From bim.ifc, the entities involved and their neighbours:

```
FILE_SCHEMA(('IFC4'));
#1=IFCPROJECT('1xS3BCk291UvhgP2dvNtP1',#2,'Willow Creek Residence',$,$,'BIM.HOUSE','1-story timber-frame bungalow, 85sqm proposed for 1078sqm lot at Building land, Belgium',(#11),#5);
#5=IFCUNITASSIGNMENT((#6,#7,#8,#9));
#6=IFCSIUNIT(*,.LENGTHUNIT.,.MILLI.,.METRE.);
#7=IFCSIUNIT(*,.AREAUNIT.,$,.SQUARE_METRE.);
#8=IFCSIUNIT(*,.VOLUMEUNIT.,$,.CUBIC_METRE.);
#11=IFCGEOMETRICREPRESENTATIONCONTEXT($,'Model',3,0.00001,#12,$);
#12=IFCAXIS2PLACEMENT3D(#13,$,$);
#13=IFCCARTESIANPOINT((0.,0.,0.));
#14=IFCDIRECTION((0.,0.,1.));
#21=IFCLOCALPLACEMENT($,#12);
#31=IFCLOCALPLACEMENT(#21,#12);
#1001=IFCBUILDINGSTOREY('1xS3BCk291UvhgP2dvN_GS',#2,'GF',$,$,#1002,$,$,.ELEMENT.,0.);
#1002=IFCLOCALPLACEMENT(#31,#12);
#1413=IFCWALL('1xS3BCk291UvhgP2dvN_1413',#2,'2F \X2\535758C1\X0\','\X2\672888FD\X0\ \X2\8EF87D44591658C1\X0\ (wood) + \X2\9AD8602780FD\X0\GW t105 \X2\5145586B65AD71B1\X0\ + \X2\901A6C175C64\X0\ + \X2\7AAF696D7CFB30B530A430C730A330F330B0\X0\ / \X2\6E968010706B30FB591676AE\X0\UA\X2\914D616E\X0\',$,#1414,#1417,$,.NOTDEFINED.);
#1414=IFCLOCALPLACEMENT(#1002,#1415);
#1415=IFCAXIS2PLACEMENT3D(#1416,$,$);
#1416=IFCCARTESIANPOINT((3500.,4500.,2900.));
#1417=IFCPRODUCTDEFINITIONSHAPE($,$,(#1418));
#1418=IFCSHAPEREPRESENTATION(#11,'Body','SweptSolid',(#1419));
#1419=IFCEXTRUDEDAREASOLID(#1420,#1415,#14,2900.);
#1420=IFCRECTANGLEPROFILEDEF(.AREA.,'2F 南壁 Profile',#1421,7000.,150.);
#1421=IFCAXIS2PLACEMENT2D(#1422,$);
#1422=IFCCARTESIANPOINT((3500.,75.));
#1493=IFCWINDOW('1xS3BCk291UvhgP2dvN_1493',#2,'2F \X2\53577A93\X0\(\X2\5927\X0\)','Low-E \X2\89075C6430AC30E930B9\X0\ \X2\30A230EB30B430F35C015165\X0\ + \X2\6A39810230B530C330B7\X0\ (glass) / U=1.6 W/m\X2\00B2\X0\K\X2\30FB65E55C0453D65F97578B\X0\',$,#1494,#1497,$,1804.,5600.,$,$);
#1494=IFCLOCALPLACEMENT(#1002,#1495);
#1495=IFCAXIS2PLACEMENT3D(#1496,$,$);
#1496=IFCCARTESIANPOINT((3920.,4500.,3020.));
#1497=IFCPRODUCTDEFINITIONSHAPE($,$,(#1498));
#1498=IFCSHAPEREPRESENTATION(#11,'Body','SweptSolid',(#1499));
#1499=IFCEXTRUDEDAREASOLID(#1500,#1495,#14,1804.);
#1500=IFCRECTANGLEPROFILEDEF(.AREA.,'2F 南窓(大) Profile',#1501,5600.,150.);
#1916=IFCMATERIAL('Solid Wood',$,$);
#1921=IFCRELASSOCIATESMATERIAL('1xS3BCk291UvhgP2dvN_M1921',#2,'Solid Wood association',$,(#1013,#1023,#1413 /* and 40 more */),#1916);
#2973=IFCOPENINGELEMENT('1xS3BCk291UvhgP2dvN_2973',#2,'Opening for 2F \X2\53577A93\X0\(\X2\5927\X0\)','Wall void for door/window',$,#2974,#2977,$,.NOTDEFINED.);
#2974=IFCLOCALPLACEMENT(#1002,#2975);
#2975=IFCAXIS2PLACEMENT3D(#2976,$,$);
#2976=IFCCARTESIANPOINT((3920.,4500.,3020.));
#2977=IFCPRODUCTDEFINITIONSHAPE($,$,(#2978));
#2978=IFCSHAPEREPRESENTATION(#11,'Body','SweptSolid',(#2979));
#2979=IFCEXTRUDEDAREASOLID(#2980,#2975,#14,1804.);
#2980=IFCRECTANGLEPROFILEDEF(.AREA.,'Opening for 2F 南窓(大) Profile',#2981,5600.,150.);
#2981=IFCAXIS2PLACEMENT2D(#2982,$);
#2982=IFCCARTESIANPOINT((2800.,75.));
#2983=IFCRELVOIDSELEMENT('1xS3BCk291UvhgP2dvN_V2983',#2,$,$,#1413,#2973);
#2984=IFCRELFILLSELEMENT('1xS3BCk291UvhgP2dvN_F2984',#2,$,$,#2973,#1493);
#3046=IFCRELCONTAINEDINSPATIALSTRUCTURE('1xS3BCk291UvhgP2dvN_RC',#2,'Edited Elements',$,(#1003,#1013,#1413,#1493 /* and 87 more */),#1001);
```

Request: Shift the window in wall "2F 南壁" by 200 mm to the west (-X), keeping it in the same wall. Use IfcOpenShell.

```python
import ifcopenshell
import ifcopenshell.api.geometry
import ifcopenshell.util.placement

model = ifcopenshell.open("bim.ifc")

window = model.by_guid("1xS3BCk291UvhgP2dvN_1493")
opening = window.FillsVoids[0].RelatingOpeningElement
wall = opening.VoidsElements[0].RelatingBuildingElement

wall_matrix = ifcopenshell.util.placement.get_local_placement(wall.ObjectPlacement)
shift = wall_matrix[:3, 0] * -200.0
before = ifcopenshell.util.placement.get_local_placement(window.ObjectPlacement)[:3, 3].copy()

# The window is not placed relative to its opening, so move both.
for product in (opening, window):
    matrix = ifcopenshell.util.placement.get_local_placement(product.ObjectPlacement)
    matrix[:3, 3] += shift
    ifcopenshell.api.geometry.edit_object_placement(model, product=product, matrix=matrix, is_si=False)

after = ifcopenshell.util.placement.get_local_placement(window.ObjectPlacement)[:3, 3]
print("window moved by", (after - before).round(3) + 0.0)

model.write("bim_updated.ifc")
```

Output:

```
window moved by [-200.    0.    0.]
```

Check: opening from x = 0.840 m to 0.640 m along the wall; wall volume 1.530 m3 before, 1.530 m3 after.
